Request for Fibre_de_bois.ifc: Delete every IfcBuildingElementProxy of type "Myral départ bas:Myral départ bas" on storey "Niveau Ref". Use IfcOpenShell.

First a look at what the model holds.

```python
import ifcopenshell
import ifcopenshell.util.element

model = ifcopenshell.open("Fibre_de_bois.ifc")
print(model.schema)
storey = next(s for s in model.by_type("IfcBuildingStorey") if s.Name == "Niveau Ref")
proxies = [e for e in ifcopenshell.util.element.get_decomposition(storey) if e.is_a("IfcBuildingElementProxy")]
seen = {}
for e in proxies:
    element_type = ifcopenshell.util.element.get_type(e)
    name = element_type.Name if element_type not in (None, e) else None
    seen[name] = seen.get(name, 0) + 1
for name, count in sorted(seen.items(), key=str):
    print(count, "x", name)
```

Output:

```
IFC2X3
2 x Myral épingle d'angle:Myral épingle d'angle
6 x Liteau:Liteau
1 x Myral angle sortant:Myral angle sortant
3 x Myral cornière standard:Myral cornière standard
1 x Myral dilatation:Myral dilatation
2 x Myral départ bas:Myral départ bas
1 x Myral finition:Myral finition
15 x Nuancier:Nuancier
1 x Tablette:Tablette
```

```python
import ifcopenshell
import ifcopenshell.api.root
import ifcopenshell.util.element

model = ifcopenshell.open("Fibre_de_bois.ifc")

storey = next(s for s in model.by_type("IfcBuildingStorey") if s.Name == "Niveau Ref")
proxies = [e for e in ifcopenshell.util.element.get_decomposition(storey) if e.is_a("IfcBuildingElementProxy")]
targets = [e for e in proxies if (t := ifcopenshell.util.element.get_type(e)) not in (None, e) and t.Name == "Myral départ bas:Myral départ bas"]

for e in targets:
    ifcopenshell.api.root.remove_product(model, product=e)
print(len(targets), "removed")

model.write("Fibre_de_bois_edited.ifc")
```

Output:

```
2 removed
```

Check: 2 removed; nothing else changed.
